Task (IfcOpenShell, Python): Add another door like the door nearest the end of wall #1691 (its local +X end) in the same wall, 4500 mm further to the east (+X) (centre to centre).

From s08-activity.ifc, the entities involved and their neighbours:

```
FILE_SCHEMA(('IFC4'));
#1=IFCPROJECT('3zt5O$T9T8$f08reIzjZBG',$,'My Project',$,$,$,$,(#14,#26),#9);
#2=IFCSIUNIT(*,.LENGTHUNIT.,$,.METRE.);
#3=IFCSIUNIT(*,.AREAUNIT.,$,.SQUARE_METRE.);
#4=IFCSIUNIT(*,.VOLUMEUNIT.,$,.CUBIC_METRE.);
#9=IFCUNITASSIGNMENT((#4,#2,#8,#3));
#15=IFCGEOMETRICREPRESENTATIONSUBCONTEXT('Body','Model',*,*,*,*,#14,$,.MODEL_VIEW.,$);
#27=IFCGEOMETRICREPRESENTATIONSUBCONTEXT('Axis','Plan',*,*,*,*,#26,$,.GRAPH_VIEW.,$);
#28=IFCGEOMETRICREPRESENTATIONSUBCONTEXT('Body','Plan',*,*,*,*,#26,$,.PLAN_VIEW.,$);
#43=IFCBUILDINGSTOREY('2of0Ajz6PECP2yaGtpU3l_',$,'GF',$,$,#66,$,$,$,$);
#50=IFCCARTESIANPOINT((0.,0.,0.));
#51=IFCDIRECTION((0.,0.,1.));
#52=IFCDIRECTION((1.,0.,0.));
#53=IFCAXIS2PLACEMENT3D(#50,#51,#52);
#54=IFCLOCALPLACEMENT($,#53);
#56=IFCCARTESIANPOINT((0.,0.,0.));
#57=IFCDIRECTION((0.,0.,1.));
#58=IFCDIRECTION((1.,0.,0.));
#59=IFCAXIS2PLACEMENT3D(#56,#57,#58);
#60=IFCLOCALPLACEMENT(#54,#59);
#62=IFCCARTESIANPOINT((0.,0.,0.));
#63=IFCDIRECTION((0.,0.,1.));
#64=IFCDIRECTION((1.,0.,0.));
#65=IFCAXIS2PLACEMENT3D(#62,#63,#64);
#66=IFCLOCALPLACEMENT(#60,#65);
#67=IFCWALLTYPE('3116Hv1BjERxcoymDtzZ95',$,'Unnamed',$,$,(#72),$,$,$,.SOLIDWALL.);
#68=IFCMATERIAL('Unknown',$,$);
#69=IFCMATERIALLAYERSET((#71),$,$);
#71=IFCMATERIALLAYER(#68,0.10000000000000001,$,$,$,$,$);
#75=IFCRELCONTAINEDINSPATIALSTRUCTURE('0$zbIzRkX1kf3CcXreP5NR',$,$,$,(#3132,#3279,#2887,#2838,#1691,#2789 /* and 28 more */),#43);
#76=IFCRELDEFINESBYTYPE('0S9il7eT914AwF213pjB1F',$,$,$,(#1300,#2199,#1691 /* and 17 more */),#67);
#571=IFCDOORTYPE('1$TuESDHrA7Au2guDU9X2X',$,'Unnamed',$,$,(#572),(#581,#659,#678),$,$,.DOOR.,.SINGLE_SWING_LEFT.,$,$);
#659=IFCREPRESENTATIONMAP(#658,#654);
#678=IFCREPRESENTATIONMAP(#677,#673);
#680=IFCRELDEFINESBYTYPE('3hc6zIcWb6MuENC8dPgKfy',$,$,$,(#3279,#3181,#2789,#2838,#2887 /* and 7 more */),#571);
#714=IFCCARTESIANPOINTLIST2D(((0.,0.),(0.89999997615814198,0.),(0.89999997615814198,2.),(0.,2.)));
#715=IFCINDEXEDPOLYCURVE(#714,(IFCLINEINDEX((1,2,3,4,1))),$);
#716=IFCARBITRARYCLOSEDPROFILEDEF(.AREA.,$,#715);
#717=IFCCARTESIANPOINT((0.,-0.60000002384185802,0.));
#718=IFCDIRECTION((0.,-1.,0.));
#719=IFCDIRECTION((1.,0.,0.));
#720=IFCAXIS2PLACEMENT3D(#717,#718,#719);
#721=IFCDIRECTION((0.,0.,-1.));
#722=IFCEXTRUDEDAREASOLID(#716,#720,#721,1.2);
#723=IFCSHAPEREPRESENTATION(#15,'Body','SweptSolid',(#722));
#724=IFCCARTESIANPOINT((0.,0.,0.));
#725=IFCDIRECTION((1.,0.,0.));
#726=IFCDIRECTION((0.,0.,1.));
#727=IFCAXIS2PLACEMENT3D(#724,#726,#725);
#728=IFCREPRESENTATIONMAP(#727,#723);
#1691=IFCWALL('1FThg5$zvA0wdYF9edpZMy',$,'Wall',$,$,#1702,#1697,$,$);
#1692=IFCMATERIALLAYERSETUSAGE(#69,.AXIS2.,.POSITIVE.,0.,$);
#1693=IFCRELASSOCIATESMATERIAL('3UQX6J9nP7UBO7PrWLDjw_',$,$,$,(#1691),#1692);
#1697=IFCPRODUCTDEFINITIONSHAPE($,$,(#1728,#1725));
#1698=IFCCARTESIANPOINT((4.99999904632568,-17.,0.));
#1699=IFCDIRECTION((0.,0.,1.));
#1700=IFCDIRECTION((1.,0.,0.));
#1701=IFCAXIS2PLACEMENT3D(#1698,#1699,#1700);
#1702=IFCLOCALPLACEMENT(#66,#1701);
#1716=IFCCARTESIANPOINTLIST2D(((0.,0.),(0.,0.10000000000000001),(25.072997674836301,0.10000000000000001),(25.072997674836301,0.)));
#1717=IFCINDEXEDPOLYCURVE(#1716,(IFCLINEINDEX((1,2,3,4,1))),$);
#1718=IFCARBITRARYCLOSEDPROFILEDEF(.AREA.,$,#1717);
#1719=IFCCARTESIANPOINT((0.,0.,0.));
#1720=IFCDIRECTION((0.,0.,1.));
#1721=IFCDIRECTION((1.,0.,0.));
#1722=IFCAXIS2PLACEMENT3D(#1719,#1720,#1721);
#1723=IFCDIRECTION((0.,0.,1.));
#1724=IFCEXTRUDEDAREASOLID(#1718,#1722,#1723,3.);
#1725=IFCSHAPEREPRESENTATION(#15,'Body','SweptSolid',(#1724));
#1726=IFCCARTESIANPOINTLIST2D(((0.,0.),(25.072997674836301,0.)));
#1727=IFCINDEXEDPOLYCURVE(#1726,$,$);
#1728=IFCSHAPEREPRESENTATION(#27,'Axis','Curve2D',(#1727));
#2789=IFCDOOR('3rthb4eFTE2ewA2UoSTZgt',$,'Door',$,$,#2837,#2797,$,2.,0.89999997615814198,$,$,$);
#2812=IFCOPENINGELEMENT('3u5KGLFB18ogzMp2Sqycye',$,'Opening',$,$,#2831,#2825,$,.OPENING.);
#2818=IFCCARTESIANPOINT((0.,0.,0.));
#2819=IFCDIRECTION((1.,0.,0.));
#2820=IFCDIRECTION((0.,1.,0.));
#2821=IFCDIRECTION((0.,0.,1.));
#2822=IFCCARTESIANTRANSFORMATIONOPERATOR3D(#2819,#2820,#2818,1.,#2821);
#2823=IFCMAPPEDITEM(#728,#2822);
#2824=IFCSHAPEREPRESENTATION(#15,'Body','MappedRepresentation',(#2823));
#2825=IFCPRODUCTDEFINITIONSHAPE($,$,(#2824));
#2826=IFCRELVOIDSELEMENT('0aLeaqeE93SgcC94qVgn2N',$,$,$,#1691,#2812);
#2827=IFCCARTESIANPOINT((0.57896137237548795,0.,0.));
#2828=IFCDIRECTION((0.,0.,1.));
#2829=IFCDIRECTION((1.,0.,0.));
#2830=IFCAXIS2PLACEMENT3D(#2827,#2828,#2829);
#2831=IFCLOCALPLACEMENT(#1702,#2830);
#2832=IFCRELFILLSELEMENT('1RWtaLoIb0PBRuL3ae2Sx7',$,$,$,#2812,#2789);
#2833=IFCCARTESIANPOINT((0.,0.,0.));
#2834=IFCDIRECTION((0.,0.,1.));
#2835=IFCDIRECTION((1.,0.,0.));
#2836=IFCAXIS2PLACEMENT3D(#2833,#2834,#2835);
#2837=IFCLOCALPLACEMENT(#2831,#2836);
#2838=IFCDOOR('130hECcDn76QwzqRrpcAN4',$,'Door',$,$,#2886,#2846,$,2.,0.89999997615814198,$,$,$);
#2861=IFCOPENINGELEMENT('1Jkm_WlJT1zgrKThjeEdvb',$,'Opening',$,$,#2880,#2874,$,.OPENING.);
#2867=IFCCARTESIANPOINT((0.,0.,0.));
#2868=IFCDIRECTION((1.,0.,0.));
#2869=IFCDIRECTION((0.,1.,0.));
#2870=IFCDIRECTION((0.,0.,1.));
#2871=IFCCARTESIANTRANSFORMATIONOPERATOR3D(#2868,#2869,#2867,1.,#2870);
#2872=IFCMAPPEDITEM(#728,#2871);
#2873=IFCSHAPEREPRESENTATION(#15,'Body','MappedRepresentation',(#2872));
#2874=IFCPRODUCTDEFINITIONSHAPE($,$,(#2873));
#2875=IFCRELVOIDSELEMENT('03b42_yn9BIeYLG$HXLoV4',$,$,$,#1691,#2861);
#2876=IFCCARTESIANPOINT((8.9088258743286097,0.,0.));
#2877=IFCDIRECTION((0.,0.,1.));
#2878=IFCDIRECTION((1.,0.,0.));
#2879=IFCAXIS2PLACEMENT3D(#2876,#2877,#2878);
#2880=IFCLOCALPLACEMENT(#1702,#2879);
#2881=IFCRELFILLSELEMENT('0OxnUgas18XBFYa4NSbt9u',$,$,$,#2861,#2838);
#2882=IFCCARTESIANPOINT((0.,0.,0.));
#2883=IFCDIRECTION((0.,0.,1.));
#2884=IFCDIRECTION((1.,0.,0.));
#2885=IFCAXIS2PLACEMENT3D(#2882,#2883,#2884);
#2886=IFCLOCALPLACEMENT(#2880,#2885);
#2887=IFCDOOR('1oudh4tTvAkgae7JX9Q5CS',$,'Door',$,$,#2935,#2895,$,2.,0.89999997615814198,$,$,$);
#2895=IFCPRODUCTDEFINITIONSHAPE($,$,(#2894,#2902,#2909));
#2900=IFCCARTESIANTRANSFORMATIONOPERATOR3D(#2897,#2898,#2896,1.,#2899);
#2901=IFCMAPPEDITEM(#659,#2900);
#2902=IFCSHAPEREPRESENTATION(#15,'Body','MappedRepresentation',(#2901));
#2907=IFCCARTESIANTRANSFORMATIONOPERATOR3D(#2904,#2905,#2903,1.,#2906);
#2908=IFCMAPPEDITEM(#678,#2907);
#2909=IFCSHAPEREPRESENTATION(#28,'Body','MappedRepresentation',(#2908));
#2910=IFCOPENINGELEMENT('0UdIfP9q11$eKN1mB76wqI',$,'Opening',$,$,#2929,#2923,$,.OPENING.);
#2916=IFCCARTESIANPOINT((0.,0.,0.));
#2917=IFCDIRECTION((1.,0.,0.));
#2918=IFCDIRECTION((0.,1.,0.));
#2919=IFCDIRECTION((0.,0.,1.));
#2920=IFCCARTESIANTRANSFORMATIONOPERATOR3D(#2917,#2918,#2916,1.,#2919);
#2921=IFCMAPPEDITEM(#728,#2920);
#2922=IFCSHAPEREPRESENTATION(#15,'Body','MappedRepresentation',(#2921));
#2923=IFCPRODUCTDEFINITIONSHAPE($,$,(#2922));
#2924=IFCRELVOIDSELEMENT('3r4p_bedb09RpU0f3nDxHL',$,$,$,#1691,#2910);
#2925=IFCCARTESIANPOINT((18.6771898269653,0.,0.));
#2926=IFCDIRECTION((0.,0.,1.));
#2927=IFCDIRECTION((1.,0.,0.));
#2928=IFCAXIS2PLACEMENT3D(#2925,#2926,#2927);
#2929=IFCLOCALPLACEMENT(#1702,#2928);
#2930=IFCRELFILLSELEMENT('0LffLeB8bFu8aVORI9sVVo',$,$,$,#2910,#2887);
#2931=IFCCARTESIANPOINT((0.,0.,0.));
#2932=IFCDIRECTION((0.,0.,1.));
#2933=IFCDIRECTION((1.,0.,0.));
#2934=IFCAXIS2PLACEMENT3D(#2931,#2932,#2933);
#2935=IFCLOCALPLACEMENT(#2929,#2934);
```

```python
import ifcopenshell
import ifcopenshell.api.feature
import ifcopenshell.api.geometry
import ifcopenshell.api.root
import ifcopenshell.geom
import ifcopenshell.util.element
import ifcopenshell.util.placement
import ifcopenshell.util.shape
import ifcopenshell.util.unit

model = ifcopenshell.open("s08-activity.ifc")
unit_scale = ifcopenshell.util.unit.calculate_unit_scale(model)
settings = ifcopenshell.geom.settings()


def volume(element):
    """Net volume in cubic metres, openings subtracted."""
    shape = ifcopenshell.geom.create_shape(settings, element)
    return ifcopenshell.util.shape.get_volume(shape.geometry)


door = model.by_guid("1oudh4tTvAkgae7JX9Q5CS")
opening = door.FillsVoids[0].RelatingOpeningElement
wall = opening.VoidsElements[0].RelatingBuildingElement
before = volume(wall)
shift = ifcopenshell.util.placement.get_local_placement(wall.ObjectPlacement)[:3, 0] * 4.5 / unit_scale

# copy_class copies the void relationship, type, container and properties, but no geometry.
new_opening = ifcopenshell.api.root.copy_class(model, product=opening)
new_opening.Representation = ifcopenshell.util.element.copy_deep(
    model, opening.Representation, exclude=["IfcGeometricRepresentationContext", "IfcRepresentationMap"]
)
new_door = ifcopenshell.api.root.copy_class(model, product=door)
new_door.Representation = ifcopenshell.util.element.copy_deep(
    model, door.Representation, exclude=["IfcGeometricRepresentationContext", "IfcRepresentationMap"]
)
ifcopenshell.api.feature.add_filling(model, opening=new_opening, element=new_door)

for old, new in ((opening, new_opening), (door, new_door)):
    matrix = ifcopenshell.util.placement.get_local_placement(old.ObjectPlacement)
    matrix[:3, 3] += shift
    ifcopenshell.api.geometry.edit_object_placement(model, product=new, matrix=matrix, is_si=False)

after = volume(wall)

print(f"wall volume {before:.3f} -> {after:.3f} m3")

model.write("s08-activity_edited.ifc")
```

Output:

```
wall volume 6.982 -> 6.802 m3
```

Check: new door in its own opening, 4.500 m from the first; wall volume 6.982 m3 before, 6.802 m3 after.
